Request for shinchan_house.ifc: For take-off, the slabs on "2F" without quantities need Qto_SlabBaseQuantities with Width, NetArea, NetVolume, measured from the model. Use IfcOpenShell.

First a look at what the model holds.

```python
import ifcopenshell
import ifcopenshell.util.element
import ifcopenshell.util.unit

model = ifcopenshell.open("shinchan_house.ifc")
print(model.schema)
for unit_type in ("LENGTHUNIT", "AREAUNIT", "VOLUMEUNIT"):
    print(unit_type, ifcopenshell.util.unit.calculate_unit_scale(model, unit_type))
storey = next(s for s in model.by_type("IfcBuildingStorey") if s.Name == "2F")
slabs = [e for e in ifcopenshell.util.element.get_decomposition(storey) if e.is_a("IfcSlab")]
for e in sorted(slabs, key=lambda e: e.id()):
    print(e.id(), e.is_a(), e.Name, list(ifcopenshell.util.element.get_psets(e, qtos_only=True)), sep=" | ")
```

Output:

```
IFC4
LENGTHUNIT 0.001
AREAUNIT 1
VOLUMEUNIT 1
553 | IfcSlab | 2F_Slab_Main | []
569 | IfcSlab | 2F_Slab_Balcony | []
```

```python
import ifcopenshell
import ifcopenshell.api.pset
import ifcopenshell.geom
import ifcopenshell.util.element
import ifcopenshell.util.shape
import ifcopenshell.util.unit

model = ifcopenshell.open("shinchan_house.ifc")
unit_scale = ifcopenshell.util.unit.calculate_unit_scale(model)
area_scale = ifcopenshell.util.unit.calculate_unit_scale(model, "AREAUNIT")
volume_scale = ifcopenshell.util.unit.calculate_unit_scale(model, "VOLUMEUNIT")
settings = ifcopenshell.geom.settings()

storey = next(s for s in model.by_type("IfcBuildingStorey") if s.Name == "2F")
slabs = [e for e in ifcopenshell.util.element.get_decomposition(storey) if e.is_a("IfcSlab")]

for e in sorted(slabs, key=lambda e: e.id()):
    if ifcopenshell.util.element.get_psets(e, qtos_only=True, should_inherit=False):
        continue
    # Geometry comes back in metres, in the element's own axes.
    shape = ifcopenshell.geom.create_shape(settings, e)
    values = {
        "Width": ifcopenshell.util.shape.get_z(shape.geometry) / unit_scale,
        "NetArea": ifcopenshell.util.shape.get_footprint_area(shape.geometry) / area_scale,
        "NetVolume": ifcopenshell.util.shape.get_volume(shape.geometry) / volume_scale,
    }
    qto = ifcopenshell.api.pset.add_qto(model, product=e, name="Qto_SlabBaseQuantities")
    ifcopenshell.api.pset.edit_qto(model, qto=qto, properties=values)
    print(e.id(), {k: round(v, 3) for k, v in values.items()})

model.write("shinchan_house-out.ifc")
```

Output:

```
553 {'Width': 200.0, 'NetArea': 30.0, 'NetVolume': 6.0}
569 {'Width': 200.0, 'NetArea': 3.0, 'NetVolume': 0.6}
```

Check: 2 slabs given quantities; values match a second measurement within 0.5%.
